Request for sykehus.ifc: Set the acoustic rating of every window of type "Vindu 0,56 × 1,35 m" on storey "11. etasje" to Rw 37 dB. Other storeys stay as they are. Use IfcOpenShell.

First a look at what the model holds.

```python
import ifcopenshell
import ifcopenshell.util.element

model = ifcopenshell.open("sykehus.ifc")
print(model.schema)
storey = next(s for s in model.by_type("IfcBuildingStorey") if s.Name == "11. etasje")
windows = [e for e in ifcopenshell.util.element.get_decomposition(storey) if e.is_a("IfcWindow")]
seen = {}
for e in windows:
    element_type = ifcopenshell.util.element.get_type(e)
    key = (element_type.Name if element_type != e and element_type else None, ifcopenshell.util.element.get_pset(e, "Pset_WindowCommon", "AcousticRating"))
    seen[key] = seen.get(key, 0) + 1
for (name, value), count in sorted(seen.items(), key=str):
    print(count, "x", name, "|", value)
```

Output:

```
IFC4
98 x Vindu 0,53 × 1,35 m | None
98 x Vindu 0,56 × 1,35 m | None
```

```python
import ifcopenshell
import ifcopenshell.api.pset
import ifcopenshell.util.element

model = ifcopenshell.open("sykehus.ifc")

storey = next(s for s in model.by_type("IfcBuildingStorey") if s.Name == "11. etasje")
windows = [e for e in ifcopenshell.util.element.get_decomposition(storey) if e.is_a("IfcWindow")]

count = 0
for e in windows:
    element_type = ifcopenshell.util.element.get_type(e)
    if element_type in (None, e) or element_type.Name != "Vindu 0,56 × 1,35 m":
        continue
    found = ifcopenshell.util.element.get_pset(e, "Pset_WindowCommon", should_inherit=False)
    if found:
        pset = model.by_id(found["id"])
        if len(ifcopenshell.util.element.get_elements_by_pset(pset)) > 1:
            pset = ifcopenshell.api.pset.unshare_pset(model, products=[e], pset=pset)[0]
    else:
        pset = ifcopenshell.api.pset.add_pset(model, product=e, name="Pset_WindowCommon")
    ifcopenshell.api.pset.edit_pset(model, pset=pset, properties={"AcousticRating": "Rw 37 dB"})
    count += 1

print(count, "windows updated")

model.write("sykehus_updated.ifc")
```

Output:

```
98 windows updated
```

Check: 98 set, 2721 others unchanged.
